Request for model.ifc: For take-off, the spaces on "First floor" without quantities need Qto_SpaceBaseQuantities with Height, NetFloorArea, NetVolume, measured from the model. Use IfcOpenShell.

First a look at what the model holds.

```python
import ifcopenshell
import ifcopenshell.util.element
import ifcopenshell.util.unit

model = ifcopenshell.open("model.ifc")
print(model.schema)
for unit_type in ("LENGTHUNIT", "AREAUNIT", "VOLUMEUNIT"):
    print(unit_type, ifcopenshell.util.unit.calculate_unit_scale(model, unit_type))
storey = next(s for s in model.by_type("IfcBuildingStorey") if s.Name == "First floor")
spaces = [e for e in ifcopenshell.util.element.get_decomposition(storey) if e.is_a("IfcSpace")]
for e in sorted(spaces, key=lambda e: e.id()):
    print(e.id(), e.is_a(), e.Name, list(ifcopenshell.util.element.get_psets(e, qtos_only=True)), sep=" | ")
```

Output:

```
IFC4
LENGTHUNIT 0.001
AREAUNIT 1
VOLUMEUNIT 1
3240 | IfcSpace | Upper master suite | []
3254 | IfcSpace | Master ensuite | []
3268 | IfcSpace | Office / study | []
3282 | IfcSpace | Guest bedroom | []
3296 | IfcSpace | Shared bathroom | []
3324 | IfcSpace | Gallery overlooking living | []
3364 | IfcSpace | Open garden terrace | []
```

```python
import ifcopenshell
import ifcopenshell.api.pset
import ifcopenshell.geom
import ifcopenshell.util.element
import ifcopenshell.util.shape
import ifcopenshell.util.unit

model = ifcopenshell.open("model.ifc")
unit_scale = ifcopenshell.util.unit.calculate_unit_scale(model)
area_scale = ifcopenshell.util.unit.calculate_unit_scale(model, "AREAUNIT")
volume_scale = ifcopenshell.util.unit.calculate_unit_scale(model, "VOLUMEUNIT")
settings = ifcopenshell.geom.settings()

storey = next(s for s in model.by_type("IfcBuildingStorey") if s.Name == "First floor")
spaces = [e for e in ifcopenshell.util.element.get_decomposition(storey) if e.is_a("IfcSpace")]

for e in sorted(spaces, key=lambda e: e.id()):
    if ifcopenshell.util.element.get_psets(e, qtos_only=True, should_inherit=False):
        continue
    # Geometry comes back in metres, in the element's own axes.
    shape = ifcopenshell.geom.create_shape(settings, e)
    values = {
        "Height": ifcopenshell.util.shape.get_z(shape.geometry) / unit_scale,
        "NetFloorArea": ifcopenshell.util.shape.get_footprint_area(shape.geometry) / area_scale,
        "NetVolume": ifcopenshell.util.shape.get_volume(shape.geometry) / volume_scale,
    }
    qto = ifcopenshell.api.pset.add_qto(model, product=e, name="Qto_SpaceBaseQuantities")
    ifcopenshell.api.pset.edit_qto(model, qto=qto, properties=values)
    print(e.id(), {k: round(v, 3) for k, v in values.items()})

model.write("model-out.ifc")
```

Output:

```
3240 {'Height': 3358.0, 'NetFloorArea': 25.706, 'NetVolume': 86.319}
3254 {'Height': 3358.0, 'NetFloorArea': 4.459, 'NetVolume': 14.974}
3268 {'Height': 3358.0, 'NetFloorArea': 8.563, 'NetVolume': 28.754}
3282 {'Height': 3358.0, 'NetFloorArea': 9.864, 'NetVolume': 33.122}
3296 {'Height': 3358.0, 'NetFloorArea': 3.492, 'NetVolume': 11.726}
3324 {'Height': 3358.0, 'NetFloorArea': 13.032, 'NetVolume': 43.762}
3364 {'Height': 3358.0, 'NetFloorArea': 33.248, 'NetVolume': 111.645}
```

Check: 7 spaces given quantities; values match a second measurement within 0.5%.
